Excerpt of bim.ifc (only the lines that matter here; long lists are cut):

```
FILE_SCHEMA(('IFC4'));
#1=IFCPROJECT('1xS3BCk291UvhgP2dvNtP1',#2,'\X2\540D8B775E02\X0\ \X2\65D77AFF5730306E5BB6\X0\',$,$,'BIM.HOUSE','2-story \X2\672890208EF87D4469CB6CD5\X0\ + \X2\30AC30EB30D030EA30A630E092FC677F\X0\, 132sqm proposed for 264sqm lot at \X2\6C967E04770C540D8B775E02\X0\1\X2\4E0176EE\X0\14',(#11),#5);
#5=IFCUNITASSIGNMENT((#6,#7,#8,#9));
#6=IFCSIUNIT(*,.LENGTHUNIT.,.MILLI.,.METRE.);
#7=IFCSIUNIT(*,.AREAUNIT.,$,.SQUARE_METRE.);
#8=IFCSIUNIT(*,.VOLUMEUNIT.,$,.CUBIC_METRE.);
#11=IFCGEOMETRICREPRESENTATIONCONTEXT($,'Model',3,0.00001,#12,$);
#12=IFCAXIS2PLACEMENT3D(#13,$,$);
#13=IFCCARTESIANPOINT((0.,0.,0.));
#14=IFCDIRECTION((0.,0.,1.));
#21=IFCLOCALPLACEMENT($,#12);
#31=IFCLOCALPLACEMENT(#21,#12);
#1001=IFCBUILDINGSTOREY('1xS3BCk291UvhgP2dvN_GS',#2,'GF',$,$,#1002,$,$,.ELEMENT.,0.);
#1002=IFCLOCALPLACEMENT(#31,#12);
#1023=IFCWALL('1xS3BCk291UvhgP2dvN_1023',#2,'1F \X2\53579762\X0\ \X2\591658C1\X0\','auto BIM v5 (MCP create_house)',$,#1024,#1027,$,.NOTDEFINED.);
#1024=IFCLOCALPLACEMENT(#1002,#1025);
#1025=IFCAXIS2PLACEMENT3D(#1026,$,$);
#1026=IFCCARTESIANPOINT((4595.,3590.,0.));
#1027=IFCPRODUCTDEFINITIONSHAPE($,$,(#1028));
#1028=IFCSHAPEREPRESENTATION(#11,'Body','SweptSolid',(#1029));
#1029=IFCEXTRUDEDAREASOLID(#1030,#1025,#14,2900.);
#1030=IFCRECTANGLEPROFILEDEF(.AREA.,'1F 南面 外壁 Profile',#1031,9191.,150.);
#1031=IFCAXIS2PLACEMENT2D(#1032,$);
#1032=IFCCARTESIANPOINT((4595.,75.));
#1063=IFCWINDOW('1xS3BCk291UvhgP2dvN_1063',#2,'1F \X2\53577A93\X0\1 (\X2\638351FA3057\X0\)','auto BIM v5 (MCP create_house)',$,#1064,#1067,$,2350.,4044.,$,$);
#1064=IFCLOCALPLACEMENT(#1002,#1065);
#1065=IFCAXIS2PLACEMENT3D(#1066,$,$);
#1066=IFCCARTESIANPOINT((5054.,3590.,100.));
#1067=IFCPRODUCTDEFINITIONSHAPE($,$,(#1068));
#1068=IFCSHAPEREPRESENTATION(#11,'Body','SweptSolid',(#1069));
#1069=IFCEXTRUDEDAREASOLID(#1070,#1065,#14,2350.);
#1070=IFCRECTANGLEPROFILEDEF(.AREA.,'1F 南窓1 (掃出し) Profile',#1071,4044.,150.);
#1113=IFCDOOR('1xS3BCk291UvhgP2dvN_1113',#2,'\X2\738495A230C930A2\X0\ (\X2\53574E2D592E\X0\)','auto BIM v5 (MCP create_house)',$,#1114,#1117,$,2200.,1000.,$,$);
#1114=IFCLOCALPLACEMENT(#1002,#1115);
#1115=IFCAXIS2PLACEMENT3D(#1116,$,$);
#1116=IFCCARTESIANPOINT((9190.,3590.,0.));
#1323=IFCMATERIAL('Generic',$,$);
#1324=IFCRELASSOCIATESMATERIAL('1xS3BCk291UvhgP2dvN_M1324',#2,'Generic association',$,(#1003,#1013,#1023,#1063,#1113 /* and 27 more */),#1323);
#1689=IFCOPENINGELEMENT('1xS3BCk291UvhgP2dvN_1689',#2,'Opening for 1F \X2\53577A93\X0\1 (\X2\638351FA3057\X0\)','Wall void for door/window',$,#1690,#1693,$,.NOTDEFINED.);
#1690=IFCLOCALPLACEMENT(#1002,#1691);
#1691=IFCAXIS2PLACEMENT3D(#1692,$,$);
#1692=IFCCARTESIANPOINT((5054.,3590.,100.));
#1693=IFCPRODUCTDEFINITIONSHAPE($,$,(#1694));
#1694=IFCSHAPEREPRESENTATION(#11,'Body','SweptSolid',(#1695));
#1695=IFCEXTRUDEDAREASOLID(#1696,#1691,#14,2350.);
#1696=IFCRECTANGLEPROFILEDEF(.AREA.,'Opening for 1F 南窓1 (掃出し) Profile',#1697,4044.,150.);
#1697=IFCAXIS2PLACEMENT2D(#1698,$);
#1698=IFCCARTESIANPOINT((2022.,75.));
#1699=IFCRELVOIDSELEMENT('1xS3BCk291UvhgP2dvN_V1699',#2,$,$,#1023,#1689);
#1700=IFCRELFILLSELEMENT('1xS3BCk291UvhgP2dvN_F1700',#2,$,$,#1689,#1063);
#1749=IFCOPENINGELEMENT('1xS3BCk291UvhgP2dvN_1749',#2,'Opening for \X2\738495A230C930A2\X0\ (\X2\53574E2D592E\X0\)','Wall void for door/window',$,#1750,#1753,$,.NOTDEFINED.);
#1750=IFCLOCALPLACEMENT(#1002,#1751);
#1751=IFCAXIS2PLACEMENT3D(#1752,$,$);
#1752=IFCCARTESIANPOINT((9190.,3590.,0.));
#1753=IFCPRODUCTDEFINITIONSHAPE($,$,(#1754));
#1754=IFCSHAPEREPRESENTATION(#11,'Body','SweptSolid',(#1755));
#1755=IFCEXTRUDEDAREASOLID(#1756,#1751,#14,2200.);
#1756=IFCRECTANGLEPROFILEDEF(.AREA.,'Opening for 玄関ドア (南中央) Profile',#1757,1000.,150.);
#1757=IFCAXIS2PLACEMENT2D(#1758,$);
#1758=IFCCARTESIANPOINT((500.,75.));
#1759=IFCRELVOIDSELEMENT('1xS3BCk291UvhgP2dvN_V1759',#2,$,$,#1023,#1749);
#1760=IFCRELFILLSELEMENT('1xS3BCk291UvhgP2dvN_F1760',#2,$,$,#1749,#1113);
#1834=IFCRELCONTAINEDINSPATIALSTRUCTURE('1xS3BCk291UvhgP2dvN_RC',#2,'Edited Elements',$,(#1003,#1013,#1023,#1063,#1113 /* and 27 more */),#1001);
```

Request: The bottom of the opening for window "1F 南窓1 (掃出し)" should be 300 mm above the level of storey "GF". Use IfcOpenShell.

```python
import numpy as np
import ifcopenshell
import ifcopenshell.api.geometry
import ifcopenshell.geom
import ifcopenshell.util.element
import ifcopenshell.util.placement
import ifcopenshell.util.shape
import ifcopenshell.util.unit

model = ifcopenshell.open("bim.ifc")
unit_scale = ifcopenshell.util.unit.calculate_unit_scale(model)

window = model.by_guid("1xS3BCk291UvhgP2dvN_1063")
opening = window.FillsVoids[0].RelatingOpeningElement
storey = ifcopenshell.util.element.get_container(window, ifc_class="IfcBuildingStorey")
level = ifcopenshell.util.placement.get_local_placement(storey.ObjectPlacement)[2, 3]

# The opening's origin need not be at the sill, so measure its lowest point.
shape = ifcopenshell.geom.create_shape(ifcopenshell.geom.settings(), opening)
bottom = ifcopenshell.util.shape.get_shape_bottom_elevation(shape, shape.geometry) / unit_scale
dz = level + 300.0 - bottom

shift = np.array([0.0, 0.0, dz])
# The window is not placed relative to its opening, so move both.
for product in (opening, window):
    matrix = ifcopenshell.util.placement.get_local_placement(product.ObjectPlacement)
    matrix[:3, 3] += shift
    ifcopenshell.api.geometry.edit_object_placement(model, product=product, matrix=matrix, is_si=False)

print(f"moved by {dz * unit_scale:+.3f} m")

model.write("bim_rev.ifc")
```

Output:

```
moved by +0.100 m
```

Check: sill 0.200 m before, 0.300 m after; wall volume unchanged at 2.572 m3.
